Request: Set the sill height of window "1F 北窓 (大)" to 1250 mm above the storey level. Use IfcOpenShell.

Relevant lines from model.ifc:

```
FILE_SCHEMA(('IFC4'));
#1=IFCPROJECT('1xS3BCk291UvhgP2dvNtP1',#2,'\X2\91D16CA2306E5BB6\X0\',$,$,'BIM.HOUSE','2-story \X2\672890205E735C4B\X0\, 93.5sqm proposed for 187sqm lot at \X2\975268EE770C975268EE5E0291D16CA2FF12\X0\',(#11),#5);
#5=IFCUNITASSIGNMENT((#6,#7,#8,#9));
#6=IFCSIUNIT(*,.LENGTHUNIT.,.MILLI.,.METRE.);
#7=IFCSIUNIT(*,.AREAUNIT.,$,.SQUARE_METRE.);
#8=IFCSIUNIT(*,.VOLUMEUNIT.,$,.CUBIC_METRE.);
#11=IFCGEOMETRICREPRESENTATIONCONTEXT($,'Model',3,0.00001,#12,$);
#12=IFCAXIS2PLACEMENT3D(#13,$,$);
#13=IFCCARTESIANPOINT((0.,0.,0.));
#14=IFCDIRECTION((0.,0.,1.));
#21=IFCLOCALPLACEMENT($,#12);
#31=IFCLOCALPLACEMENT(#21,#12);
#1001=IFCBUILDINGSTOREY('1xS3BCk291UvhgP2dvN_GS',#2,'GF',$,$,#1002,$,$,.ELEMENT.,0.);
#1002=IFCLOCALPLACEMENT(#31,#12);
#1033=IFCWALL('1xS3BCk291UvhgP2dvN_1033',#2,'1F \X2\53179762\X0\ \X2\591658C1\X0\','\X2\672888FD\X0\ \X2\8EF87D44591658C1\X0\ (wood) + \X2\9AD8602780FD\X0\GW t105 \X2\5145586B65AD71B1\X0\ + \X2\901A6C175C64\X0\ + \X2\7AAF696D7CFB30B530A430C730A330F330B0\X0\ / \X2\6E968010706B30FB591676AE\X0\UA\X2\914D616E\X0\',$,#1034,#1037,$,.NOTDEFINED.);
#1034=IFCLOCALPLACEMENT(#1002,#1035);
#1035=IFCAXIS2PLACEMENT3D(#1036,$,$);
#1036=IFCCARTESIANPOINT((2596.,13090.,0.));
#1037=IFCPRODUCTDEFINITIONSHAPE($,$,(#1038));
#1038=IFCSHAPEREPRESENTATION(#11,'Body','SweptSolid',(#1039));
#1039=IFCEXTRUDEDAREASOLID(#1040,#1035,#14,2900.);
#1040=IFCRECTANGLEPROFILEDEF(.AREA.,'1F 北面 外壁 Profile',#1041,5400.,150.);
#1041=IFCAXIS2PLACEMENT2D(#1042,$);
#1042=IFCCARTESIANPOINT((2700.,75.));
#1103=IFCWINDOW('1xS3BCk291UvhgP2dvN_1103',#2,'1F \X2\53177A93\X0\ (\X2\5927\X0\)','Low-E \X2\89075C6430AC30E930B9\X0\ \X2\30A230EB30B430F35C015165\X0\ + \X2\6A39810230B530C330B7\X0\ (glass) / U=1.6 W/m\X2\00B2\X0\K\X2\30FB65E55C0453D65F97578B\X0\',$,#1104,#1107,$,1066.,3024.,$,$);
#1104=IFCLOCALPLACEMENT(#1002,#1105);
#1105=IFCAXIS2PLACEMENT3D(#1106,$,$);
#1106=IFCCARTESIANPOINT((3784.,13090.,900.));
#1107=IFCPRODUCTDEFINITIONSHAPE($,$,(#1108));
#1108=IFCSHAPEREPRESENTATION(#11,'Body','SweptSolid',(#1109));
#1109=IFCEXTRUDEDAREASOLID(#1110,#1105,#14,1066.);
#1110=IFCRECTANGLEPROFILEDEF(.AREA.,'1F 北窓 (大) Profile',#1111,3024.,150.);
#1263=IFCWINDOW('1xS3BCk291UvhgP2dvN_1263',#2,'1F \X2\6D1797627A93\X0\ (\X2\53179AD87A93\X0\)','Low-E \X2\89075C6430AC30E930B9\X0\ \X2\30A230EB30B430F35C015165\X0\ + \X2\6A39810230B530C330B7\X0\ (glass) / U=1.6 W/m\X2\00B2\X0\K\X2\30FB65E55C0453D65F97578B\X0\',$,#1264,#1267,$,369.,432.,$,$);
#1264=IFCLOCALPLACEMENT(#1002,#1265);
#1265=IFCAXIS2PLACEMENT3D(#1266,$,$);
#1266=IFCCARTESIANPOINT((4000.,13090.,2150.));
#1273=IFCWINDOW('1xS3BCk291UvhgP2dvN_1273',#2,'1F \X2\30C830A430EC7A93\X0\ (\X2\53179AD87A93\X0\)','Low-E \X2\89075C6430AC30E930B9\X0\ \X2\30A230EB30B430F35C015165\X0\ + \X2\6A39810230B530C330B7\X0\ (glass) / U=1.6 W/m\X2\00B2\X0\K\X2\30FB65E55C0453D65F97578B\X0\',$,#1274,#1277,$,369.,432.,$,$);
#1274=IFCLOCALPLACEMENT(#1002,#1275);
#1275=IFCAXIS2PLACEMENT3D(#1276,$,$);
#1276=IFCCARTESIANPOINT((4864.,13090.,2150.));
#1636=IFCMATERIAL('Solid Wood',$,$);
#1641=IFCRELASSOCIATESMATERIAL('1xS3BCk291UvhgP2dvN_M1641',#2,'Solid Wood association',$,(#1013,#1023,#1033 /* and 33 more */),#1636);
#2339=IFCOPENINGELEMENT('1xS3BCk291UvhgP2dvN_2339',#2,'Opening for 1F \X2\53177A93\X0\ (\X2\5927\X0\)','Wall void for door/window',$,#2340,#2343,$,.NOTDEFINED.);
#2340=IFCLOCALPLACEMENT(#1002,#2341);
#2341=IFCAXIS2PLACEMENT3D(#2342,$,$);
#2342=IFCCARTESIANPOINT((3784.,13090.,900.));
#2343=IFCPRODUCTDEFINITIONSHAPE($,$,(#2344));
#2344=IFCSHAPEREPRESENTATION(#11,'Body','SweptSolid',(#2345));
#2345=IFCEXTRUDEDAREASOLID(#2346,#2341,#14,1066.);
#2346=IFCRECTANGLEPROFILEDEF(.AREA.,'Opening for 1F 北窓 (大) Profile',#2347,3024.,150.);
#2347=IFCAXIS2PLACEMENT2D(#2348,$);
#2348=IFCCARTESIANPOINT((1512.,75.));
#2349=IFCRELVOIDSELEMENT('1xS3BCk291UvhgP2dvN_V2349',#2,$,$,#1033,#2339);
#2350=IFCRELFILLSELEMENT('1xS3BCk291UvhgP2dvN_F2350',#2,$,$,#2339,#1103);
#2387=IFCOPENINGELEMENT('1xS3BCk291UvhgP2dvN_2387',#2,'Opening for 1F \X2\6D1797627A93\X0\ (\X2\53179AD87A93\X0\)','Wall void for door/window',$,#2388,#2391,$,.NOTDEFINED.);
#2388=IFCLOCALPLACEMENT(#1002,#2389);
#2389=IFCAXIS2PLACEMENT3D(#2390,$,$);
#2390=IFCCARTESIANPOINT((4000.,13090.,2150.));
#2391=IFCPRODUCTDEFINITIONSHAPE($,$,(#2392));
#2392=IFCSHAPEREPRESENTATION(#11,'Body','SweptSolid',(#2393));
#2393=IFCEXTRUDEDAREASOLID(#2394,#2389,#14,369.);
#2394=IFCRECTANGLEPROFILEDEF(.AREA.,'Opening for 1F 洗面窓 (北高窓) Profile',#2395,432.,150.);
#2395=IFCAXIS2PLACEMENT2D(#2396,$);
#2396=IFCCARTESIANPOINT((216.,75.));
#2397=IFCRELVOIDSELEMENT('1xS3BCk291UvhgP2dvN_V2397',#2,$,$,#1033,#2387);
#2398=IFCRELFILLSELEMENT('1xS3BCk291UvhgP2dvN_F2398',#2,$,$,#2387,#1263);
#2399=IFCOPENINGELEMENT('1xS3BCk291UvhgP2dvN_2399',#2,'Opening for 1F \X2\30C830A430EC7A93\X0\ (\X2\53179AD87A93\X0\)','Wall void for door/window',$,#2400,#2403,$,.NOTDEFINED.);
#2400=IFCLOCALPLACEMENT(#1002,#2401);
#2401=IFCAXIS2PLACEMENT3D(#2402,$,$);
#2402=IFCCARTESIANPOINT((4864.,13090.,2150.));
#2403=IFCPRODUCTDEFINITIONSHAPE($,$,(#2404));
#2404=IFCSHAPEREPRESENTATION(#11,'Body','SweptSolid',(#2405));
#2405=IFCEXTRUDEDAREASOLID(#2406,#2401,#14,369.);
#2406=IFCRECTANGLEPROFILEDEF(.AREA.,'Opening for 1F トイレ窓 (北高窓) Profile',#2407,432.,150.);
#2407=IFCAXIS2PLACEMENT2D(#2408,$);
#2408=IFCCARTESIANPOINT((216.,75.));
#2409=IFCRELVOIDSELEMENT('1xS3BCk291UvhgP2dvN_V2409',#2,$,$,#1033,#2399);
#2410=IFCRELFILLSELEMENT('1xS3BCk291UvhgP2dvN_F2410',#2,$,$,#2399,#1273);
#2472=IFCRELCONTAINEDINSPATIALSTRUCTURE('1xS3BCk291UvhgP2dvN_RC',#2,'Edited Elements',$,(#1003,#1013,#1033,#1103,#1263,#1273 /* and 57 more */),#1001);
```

```python
import numpy as np
import ifcopenshell
import ifcopenshell.api.geometry
import ifcopenshell.geom
import ifcopenshell.util.element
import ifcopenshell.util.placement
import ifcopenshell.util.shape
import ifcopenshell.util.unit

model = ifcopenshell.open("model.ifc")
unit_scale = ifcopenshell.util.unit.calculate_unit_scale(model)

window = model.by_id(1103)
opening = window.FillsVoids[0].RelatingOpeningElement
storey = ifcopenshell.util.element.get_container(window, ifc_class="IfcBuildingStorey")
level = ifcopenshell.util.placement.get_local_placement(storey.ObjectPlacement)[2, 3]

# The opening's origin need not be at the sill, so measure its lowest point.
shape = ifcopenshell.geom.create_shape(ifcopenshell.geom.settings(), opening)
bottom = ifcopenshell.util.shape.get_shape_bottom_elevation(shape, shape.geometry) / unit_scale
dz = level + 1.25 / unit_scale - bottom

shift = np.array([0.0, 0.0, dz])
# The window is not placed relative to its opening, so move both.
for product in (opening, window):
    matrix = ifcopenshell.util.placement.get_local_placement(product.ObjectPlacement)
    matrix[:3, 3] += shift
    ifcopenshell.api.geometry.edit_object_placement(model, product=product, matrix=matrix, is_si=False)

print(f"moved by {dz * unit_scale:+.3f} m")

model.write("model_updated.ifc")
```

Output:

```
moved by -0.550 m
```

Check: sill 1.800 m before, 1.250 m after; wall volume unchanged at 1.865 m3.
